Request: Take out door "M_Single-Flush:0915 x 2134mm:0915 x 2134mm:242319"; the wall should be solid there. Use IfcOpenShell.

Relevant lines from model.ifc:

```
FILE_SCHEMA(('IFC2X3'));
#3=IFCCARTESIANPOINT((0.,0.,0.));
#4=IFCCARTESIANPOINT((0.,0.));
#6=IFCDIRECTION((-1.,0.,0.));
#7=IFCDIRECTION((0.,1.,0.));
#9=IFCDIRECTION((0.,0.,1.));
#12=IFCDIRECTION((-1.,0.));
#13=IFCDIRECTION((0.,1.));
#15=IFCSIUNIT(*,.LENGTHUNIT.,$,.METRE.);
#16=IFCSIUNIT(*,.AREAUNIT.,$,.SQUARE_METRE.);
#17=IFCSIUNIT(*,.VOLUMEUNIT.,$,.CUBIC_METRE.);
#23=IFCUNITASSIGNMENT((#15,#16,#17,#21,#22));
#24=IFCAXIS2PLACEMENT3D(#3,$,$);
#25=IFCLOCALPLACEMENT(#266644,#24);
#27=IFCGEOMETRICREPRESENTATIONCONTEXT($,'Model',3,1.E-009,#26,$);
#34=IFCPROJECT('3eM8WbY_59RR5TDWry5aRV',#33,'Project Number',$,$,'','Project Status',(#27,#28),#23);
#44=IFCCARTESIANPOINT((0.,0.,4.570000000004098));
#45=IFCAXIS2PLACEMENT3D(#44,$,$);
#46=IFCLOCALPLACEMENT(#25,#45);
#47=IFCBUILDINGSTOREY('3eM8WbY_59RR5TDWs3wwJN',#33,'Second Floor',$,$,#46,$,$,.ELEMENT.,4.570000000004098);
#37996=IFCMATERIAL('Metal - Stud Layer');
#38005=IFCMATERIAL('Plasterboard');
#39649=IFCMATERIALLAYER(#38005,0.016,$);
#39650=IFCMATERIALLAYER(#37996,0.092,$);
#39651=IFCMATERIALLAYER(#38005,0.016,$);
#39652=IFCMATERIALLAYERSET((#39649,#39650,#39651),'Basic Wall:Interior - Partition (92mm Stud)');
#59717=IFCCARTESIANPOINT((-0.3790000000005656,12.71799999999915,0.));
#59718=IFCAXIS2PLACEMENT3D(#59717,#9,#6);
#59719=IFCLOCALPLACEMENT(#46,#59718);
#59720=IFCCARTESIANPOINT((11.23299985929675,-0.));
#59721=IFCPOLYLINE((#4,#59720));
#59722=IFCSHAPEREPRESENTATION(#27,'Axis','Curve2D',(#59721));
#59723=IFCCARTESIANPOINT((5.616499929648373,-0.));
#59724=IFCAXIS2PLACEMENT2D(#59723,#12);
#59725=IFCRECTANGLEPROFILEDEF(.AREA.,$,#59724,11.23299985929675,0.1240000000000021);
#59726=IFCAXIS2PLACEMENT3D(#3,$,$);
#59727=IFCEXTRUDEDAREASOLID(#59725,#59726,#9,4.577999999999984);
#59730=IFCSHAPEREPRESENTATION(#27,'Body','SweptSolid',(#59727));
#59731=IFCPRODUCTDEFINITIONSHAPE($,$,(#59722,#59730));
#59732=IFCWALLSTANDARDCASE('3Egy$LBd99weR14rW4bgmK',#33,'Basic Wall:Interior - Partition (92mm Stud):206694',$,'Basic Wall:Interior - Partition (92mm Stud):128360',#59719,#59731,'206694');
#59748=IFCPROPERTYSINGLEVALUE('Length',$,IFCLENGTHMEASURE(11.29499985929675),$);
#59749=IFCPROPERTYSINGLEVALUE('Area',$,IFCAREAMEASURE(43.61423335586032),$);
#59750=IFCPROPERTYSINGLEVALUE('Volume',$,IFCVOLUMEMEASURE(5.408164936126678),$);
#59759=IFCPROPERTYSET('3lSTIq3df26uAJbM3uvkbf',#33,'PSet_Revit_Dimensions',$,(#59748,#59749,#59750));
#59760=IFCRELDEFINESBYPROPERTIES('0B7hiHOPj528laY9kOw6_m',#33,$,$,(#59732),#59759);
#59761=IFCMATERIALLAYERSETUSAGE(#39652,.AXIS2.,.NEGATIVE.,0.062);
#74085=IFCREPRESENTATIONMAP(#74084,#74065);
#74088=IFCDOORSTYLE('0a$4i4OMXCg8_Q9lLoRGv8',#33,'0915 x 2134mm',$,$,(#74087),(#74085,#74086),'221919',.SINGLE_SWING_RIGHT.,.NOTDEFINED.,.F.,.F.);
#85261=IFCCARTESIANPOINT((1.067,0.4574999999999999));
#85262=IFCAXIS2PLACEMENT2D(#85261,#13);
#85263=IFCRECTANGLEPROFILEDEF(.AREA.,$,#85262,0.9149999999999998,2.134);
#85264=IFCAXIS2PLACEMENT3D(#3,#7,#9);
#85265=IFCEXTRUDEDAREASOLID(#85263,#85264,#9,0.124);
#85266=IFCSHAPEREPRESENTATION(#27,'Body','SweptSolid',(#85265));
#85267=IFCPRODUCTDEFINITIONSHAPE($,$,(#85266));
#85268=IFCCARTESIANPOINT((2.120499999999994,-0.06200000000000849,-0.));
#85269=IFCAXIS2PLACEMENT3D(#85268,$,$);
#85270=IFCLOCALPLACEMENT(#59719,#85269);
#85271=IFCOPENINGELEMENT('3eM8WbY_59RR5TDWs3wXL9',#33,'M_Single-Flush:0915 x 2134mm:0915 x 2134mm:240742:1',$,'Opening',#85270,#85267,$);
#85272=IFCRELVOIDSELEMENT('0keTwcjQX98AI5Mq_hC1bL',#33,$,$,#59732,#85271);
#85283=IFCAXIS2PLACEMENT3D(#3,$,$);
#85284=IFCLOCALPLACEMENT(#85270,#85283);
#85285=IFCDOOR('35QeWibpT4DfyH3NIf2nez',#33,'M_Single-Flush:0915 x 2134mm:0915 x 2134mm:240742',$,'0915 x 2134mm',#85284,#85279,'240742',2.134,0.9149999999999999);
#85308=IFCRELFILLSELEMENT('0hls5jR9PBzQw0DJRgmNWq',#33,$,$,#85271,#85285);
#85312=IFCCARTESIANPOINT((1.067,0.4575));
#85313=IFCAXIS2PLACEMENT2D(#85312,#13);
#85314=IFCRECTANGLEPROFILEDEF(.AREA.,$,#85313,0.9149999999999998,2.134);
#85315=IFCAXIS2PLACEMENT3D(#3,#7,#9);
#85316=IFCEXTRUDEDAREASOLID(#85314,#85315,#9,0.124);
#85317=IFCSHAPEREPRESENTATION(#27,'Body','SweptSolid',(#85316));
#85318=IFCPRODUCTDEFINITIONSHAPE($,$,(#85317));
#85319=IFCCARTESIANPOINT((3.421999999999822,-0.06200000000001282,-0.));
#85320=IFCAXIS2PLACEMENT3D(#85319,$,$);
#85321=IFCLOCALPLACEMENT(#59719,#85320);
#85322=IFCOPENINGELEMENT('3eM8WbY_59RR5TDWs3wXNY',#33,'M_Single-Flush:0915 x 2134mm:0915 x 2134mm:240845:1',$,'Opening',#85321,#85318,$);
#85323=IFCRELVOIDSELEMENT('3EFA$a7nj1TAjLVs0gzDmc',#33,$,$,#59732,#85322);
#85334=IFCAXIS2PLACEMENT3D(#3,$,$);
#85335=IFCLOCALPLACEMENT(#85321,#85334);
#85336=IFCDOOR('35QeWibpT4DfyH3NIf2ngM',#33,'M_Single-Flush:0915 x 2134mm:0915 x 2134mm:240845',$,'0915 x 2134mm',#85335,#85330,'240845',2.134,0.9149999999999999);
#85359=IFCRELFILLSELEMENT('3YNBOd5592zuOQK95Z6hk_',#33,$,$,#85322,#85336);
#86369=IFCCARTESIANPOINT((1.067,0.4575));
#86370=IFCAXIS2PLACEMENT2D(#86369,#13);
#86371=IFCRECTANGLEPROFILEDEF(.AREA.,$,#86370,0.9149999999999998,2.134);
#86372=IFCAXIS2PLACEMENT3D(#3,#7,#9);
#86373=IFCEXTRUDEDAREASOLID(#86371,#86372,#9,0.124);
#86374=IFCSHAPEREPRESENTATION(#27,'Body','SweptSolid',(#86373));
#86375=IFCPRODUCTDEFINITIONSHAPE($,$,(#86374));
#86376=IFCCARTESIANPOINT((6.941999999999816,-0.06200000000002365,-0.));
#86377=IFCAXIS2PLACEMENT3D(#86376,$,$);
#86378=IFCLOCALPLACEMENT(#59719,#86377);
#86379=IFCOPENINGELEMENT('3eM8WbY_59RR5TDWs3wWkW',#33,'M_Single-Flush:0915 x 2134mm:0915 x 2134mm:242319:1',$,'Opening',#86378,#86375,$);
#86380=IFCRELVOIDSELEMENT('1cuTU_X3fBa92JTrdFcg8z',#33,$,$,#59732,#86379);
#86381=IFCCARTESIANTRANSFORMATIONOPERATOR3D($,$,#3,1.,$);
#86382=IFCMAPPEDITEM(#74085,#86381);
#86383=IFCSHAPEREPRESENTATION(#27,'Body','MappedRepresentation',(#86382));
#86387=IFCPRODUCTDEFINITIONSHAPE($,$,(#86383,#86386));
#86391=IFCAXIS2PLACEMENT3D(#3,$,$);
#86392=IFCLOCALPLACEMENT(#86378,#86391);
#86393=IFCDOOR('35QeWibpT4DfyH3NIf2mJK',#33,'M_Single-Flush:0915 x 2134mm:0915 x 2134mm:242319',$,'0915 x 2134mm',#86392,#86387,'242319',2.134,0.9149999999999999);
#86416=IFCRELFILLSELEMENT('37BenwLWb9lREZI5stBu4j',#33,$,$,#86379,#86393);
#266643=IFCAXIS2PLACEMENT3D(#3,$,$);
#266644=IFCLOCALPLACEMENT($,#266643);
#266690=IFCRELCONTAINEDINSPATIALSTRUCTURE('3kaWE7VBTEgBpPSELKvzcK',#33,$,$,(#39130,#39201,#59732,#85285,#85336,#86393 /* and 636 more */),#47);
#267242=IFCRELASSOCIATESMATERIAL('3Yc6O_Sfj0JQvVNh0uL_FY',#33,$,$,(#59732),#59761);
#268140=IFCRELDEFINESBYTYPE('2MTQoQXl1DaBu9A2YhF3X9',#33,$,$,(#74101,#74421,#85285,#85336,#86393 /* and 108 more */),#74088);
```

```python
import ifcopenshell
import ifcopenshell.api.feature
import ifcopenshell.api.pset
import ifcopenshell.api.root
import ifcopenshell.geom
import ifcopenshell.util.element
import ifcopenshell.util.shape
import ifcopenshell.util.unit

model = ifcopenshell.open("model.ifc")
area_scale = ifcopenshell.util.unit.calculate_unit_scale(model, "AREAUNIT")
volume_scale = ifcopenshell.util.unit.calculate_unit_scale(model, "VOLUMEUNIT")
settings = ifcopenshell.geom.settings()


def volume(element):
    """Net volume in cubic metres, openings subtracted."""
    shape = ifcopenshell.geom.create_shape(settings, element)
    return ifcopenshell.util.shape.get_volume(shape.geometry)


door = model.by_guid("35QeWibpT4DfyH3NIf2mJK")
opening = door.FillsVoids[0].RelatingOpeningElement
wall = opening.VoidsElements[0].RelatingBuildingElement
before = volume(wall)

ifcopenshell.api.root.remove_product(model, product=door)
ifcopenshell.api.feature.remove_feature(model, feature=opening)

after = volume(wall)
thickness = 0.124  # wall thickness in metres

# Update the wall's stored quantities.
pset = model.by_id(ifcopenshell.util.element.get_pset(wall, "PSet_Revit_Dimensions", should_inherit=False)["id"])
ifcopenshell.api.pset.edit_pset(model, pset=pset, properties={
    "Area": model.create_entity("IfcAreaMeasure", after / thickness / area_scale),
    "Volume": model.create_entity("IfcVolumeMeasure", after / volume_scale),
})

print(f"wall volume {before:.3f} -> {after:.3f} m3")

model.write("model_updated.ifc")
```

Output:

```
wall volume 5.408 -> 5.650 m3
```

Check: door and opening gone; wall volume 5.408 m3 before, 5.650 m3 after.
